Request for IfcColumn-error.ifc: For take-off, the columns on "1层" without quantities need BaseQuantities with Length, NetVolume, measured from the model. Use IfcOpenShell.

First a look at what the model holds.

```python
import ifcopenshell
import ifcopenshell.util.element
import ifcopenshell.util.unit

model = ifcopenshell.open("IfcColumn-error.ifc")
print(model.schema)
for unit_type in ("LENGTHUNIT", "AREAUNIT", "VOLUMEUNIT"):
    print(unit_type, ifcopenshell.util.unit.calculate_unit_scale(model, unit_type))
storey = next(s for s in model.by_type("IfcBuildingStorey") if s.Name == "1层")
columns = [e for e in ifcopenshell.util.element.get_decomposition(storey) if e.is_a("IfcColumn")]
for e in sorted(columns, key=lambda e: e.id()):
    print(e.id(), e.is_a(), e.Name, list(ifcopenshell.util.element.get_psets(e, qtos_only=True)), sep=" | ")
```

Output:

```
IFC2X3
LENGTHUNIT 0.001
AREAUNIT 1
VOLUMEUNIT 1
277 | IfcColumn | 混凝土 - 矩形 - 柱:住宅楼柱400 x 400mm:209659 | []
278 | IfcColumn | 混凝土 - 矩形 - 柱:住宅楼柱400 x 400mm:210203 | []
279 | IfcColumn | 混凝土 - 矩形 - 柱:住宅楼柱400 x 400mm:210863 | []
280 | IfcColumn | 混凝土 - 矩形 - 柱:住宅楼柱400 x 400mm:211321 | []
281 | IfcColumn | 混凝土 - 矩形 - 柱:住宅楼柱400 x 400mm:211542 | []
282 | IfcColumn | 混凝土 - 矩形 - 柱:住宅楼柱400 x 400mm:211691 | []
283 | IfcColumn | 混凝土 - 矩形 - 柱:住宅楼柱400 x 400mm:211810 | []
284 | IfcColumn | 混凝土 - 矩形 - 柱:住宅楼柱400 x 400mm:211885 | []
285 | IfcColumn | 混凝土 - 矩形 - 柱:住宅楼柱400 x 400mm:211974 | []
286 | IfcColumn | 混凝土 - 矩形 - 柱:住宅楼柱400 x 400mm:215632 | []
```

```python
import ifcopenshell
import ifcopenshell.api.pset
import ifcopenshell.geom
import ifcopenshell.util.element
import ifcopenshell.util.shape
import ifcopenshell.util.unit

model = ifcopenshell.open("IfcColumn-error.ifc")
unit_scale = ifcopenshell.util.unit.calculate_unit_scale(model)
volume_scale = ifcopenshell.util.unit.calculate_unit_scale(model, "VOLUMEUNIT")
settings = ifcopenshell.geom.settings()

storey = next(s for s in model.by_type("IfcBuildingStorey") if s.Name == "1层")
columns = [e for e in ifcopenshell.util.element.get_decomposition(storey) if e.is_a("IfcColumn")]

for e in sorted(columns, key=lambda e: e.id()):
    if ifcopenshell.util.element.get_psets(e, qtos_only=True, should_inherit=False):
        continue
    # Geometry comes back in metres, in the element's own axes.
    shape = ifcopenshell.geom.create_shape(settings, e)
    values = {
        "Length": ifcopenshell.util.shape.get_z(shape.geometry) / unit_scale,
        "NetVolume": ifcopenshell.util.shape.get_volume(shape.geometry) / volume_scale,
    }
    qto = ifcopenshell.api.pset.add_qto(model, product=e, name="BaseQuantities")
    ifcopenshell.api.pset.edit_qto(model, qto=qto, properties=values)
    print(e.id(), {k: round(v, 3) for k, v in values.items()})

model.write("IfcColumn-error_rev.ifc")
```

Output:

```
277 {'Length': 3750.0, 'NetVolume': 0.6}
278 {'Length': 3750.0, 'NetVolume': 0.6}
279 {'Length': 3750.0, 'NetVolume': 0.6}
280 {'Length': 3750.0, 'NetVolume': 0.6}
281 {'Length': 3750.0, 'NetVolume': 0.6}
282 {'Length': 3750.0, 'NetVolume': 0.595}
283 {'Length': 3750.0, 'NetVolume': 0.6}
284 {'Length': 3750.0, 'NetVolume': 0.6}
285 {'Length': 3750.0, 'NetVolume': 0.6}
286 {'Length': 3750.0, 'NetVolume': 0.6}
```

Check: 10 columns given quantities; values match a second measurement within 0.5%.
